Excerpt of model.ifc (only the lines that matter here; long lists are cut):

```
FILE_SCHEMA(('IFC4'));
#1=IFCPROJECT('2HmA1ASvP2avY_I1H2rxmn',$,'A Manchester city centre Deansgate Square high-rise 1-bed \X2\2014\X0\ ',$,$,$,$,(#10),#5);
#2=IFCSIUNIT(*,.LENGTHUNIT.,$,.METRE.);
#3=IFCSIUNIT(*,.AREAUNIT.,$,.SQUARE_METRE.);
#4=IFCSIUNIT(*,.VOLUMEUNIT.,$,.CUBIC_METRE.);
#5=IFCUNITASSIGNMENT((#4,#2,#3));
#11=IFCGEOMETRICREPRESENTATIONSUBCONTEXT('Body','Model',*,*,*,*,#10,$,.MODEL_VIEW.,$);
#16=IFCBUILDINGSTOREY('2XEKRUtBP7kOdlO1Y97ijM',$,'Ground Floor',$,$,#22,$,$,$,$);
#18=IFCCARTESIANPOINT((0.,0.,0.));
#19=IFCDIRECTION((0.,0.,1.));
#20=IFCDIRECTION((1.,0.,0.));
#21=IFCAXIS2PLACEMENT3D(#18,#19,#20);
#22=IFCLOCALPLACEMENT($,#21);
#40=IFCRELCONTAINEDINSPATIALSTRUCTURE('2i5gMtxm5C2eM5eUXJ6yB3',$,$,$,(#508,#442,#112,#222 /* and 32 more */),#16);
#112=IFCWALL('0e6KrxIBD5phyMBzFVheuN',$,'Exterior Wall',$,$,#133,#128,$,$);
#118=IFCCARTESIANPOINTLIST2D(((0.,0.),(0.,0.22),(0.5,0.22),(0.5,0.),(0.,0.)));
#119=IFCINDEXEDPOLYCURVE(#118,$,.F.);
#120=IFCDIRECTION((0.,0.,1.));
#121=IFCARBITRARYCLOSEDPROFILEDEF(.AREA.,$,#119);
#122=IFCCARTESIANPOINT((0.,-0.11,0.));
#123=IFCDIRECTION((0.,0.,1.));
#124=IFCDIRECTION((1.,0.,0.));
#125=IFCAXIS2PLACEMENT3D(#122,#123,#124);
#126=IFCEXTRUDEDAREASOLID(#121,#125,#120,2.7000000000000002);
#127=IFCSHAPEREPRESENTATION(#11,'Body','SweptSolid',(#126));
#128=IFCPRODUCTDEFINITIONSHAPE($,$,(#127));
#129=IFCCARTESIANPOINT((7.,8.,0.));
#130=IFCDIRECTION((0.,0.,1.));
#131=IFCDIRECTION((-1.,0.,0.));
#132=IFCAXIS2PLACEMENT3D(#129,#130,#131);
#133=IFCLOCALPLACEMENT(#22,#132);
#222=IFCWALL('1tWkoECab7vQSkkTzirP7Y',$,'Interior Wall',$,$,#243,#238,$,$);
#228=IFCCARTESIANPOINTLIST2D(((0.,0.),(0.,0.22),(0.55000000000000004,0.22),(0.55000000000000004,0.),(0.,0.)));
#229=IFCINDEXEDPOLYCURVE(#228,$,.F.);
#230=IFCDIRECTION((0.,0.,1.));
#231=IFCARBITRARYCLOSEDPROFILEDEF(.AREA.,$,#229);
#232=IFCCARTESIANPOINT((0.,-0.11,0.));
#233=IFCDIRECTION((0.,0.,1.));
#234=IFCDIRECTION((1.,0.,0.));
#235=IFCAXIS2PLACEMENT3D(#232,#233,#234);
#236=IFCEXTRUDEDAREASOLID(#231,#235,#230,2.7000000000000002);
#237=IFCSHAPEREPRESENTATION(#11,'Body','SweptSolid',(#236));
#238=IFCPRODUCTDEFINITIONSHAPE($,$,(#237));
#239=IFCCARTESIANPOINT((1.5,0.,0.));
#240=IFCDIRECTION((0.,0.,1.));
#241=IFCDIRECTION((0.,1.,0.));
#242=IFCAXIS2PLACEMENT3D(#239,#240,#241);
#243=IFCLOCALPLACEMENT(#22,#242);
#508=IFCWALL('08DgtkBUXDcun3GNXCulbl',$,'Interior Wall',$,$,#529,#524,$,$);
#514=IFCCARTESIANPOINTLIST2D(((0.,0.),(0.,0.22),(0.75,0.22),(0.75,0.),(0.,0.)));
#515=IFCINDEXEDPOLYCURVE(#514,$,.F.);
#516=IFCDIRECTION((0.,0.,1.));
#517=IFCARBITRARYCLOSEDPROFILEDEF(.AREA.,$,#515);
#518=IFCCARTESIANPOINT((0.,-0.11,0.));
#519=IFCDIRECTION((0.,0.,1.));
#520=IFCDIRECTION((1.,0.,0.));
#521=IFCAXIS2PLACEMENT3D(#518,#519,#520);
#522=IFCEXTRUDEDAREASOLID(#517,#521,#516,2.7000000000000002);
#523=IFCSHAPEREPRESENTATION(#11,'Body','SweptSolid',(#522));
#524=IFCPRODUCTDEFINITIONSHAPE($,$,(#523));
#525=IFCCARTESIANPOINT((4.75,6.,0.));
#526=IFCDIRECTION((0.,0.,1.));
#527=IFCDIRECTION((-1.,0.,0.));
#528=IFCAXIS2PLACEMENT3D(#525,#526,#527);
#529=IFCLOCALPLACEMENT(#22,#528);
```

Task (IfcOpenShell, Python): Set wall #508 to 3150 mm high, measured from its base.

```python
import ifcopenshell
import ifcopenshell.geom
import ifcopenshell.util.representation
import ifcopenshell.util.shape

model = ifcopenshell.open("model.ifc")
settings = ifcopenshell.geom.settings()


def volume(element):
    """Net volume in cubic metres, openings subtracted."""
    shape = ifcopenshell.geom.create_shape(settings, element)
    return ifcopenshell.util.shape.get_volume(shape.geometry)


wall = model.by_id(508)
before = volume(wall)

body = ifcopenshell.util.representation.get_representation(wall, "Model", "Body")
solid = body.Items[0]
old_height = solid.Depth
solid.Depth = 3.15
after = volume(wall)

print(f"height {old_height:g} -> {solid.Depth:g}, volume {before:.3f} -> {after:.3f} m3")

model.write("model_updated.ifc")
```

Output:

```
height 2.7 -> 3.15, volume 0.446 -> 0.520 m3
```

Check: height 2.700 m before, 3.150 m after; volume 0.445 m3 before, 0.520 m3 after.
